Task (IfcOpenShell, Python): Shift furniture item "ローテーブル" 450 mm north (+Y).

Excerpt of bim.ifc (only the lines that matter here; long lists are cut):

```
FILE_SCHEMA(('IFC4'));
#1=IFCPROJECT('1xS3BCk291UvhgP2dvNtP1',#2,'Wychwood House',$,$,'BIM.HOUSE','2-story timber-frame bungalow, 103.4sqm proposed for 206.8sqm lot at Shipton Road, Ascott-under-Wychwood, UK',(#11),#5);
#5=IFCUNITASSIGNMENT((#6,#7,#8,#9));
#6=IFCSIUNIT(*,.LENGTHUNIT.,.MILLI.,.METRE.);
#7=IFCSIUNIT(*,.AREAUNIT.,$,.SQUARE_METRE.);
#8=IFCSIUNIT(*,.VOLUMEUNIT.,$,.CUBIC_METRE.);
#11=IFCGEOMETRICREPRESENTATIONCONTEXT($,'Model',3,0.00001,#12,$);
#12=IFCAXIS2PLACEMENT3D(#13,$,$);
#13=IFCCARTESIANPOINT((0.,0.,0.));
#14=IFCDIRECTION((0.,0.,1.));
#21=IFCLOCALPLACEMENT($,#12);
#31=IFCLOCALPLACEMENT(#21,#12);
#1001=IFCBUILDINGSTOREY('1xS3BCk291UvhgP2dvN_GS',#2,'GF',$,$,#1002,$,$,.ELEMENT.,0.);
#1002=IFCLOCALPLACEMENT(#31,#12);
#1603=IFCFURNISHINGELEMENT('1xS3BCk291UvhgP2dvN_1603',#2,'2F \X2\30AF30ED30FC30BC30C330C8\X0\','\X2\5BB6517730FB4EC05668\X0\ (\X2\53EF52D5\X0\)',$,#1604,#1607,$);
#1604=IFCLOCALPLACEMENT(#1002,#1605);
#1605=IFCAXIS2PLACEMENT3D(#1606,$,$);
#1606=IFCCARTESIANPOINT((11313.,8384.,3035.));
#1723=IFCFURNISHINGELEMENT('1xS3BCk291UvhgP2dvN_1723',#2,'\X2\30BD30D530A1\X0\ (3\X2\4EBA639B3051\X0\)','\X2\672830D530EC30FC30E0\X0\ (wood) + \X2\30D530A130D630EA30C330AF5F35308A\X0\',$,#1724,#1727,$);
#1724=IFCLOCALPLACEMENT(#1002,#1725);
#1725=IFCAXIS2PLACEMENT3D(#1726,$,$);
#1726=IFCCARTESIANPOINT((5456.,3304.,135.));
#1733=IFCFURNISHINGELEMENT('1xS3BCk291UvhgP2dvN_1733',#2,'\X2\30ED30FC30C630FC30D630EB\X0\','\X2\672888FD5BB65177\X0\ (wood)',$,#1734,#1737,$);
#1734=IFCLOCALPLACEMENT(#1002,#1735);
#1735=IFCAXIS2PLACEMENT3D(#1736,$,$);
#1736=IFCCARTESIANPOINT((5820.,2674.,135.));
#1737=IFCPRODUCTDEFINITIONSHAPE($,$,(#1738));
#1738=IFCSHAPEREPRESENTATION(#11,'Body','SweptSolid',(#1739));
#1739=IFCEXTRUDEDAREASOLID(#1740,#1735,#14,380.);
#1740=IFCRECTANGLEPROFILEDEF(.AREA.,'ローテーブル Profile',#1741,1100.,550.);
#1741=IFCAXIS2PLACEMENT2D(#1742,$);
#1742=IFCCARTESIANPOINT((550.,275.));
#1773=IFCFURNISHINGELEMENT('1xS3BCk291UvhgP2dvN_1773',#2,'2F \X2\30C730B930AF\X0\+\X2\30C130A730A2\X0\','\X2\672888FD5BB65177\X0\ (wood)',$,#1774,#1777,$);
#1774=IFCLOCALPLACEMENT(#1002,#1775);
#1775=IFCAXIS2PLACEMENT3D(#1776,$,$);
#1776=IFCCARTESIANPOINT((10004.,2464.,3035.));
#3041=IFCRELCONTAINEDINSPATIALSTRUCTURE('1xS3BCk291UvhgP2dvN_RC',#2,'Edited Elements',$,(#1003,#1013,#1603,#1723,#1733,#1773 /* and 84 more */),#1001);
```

```python
import ifcopenshell
import ifcopenshell.api.geometry
import ifcopenshell.util.placement
import ifcopenshell.util.unit

model = ifcopenshell.open("bim.ifc")
unit_scale = ifcopenshell.util.unit.calculate_unit_scale(model)

item = model.by_guid("1xS3BCk291UvhgP2dvN_1733")
matrix = ifcopenshell.util.placement.get_local_placement(item.ObjectPlacement)
matrix[1, 3] += 0.45 / unit_scale
ifcopenshell.api.geometry.edit_object_placement(model, product=item, matrix=matrix, is_si=False)

print(ifcopenshell.util.placement.get_local_placement(item.ObjectPlacement).round(3) + 0.0)

model.write("bim_rev.ifc")
```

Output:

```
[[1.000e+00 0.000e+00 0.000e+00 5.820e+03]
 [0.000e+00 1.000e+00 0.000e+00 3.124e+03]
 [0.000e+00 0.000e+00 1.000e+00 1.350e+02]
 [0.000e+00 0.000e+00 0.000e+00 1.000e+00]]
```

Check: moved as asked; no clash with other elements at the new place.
